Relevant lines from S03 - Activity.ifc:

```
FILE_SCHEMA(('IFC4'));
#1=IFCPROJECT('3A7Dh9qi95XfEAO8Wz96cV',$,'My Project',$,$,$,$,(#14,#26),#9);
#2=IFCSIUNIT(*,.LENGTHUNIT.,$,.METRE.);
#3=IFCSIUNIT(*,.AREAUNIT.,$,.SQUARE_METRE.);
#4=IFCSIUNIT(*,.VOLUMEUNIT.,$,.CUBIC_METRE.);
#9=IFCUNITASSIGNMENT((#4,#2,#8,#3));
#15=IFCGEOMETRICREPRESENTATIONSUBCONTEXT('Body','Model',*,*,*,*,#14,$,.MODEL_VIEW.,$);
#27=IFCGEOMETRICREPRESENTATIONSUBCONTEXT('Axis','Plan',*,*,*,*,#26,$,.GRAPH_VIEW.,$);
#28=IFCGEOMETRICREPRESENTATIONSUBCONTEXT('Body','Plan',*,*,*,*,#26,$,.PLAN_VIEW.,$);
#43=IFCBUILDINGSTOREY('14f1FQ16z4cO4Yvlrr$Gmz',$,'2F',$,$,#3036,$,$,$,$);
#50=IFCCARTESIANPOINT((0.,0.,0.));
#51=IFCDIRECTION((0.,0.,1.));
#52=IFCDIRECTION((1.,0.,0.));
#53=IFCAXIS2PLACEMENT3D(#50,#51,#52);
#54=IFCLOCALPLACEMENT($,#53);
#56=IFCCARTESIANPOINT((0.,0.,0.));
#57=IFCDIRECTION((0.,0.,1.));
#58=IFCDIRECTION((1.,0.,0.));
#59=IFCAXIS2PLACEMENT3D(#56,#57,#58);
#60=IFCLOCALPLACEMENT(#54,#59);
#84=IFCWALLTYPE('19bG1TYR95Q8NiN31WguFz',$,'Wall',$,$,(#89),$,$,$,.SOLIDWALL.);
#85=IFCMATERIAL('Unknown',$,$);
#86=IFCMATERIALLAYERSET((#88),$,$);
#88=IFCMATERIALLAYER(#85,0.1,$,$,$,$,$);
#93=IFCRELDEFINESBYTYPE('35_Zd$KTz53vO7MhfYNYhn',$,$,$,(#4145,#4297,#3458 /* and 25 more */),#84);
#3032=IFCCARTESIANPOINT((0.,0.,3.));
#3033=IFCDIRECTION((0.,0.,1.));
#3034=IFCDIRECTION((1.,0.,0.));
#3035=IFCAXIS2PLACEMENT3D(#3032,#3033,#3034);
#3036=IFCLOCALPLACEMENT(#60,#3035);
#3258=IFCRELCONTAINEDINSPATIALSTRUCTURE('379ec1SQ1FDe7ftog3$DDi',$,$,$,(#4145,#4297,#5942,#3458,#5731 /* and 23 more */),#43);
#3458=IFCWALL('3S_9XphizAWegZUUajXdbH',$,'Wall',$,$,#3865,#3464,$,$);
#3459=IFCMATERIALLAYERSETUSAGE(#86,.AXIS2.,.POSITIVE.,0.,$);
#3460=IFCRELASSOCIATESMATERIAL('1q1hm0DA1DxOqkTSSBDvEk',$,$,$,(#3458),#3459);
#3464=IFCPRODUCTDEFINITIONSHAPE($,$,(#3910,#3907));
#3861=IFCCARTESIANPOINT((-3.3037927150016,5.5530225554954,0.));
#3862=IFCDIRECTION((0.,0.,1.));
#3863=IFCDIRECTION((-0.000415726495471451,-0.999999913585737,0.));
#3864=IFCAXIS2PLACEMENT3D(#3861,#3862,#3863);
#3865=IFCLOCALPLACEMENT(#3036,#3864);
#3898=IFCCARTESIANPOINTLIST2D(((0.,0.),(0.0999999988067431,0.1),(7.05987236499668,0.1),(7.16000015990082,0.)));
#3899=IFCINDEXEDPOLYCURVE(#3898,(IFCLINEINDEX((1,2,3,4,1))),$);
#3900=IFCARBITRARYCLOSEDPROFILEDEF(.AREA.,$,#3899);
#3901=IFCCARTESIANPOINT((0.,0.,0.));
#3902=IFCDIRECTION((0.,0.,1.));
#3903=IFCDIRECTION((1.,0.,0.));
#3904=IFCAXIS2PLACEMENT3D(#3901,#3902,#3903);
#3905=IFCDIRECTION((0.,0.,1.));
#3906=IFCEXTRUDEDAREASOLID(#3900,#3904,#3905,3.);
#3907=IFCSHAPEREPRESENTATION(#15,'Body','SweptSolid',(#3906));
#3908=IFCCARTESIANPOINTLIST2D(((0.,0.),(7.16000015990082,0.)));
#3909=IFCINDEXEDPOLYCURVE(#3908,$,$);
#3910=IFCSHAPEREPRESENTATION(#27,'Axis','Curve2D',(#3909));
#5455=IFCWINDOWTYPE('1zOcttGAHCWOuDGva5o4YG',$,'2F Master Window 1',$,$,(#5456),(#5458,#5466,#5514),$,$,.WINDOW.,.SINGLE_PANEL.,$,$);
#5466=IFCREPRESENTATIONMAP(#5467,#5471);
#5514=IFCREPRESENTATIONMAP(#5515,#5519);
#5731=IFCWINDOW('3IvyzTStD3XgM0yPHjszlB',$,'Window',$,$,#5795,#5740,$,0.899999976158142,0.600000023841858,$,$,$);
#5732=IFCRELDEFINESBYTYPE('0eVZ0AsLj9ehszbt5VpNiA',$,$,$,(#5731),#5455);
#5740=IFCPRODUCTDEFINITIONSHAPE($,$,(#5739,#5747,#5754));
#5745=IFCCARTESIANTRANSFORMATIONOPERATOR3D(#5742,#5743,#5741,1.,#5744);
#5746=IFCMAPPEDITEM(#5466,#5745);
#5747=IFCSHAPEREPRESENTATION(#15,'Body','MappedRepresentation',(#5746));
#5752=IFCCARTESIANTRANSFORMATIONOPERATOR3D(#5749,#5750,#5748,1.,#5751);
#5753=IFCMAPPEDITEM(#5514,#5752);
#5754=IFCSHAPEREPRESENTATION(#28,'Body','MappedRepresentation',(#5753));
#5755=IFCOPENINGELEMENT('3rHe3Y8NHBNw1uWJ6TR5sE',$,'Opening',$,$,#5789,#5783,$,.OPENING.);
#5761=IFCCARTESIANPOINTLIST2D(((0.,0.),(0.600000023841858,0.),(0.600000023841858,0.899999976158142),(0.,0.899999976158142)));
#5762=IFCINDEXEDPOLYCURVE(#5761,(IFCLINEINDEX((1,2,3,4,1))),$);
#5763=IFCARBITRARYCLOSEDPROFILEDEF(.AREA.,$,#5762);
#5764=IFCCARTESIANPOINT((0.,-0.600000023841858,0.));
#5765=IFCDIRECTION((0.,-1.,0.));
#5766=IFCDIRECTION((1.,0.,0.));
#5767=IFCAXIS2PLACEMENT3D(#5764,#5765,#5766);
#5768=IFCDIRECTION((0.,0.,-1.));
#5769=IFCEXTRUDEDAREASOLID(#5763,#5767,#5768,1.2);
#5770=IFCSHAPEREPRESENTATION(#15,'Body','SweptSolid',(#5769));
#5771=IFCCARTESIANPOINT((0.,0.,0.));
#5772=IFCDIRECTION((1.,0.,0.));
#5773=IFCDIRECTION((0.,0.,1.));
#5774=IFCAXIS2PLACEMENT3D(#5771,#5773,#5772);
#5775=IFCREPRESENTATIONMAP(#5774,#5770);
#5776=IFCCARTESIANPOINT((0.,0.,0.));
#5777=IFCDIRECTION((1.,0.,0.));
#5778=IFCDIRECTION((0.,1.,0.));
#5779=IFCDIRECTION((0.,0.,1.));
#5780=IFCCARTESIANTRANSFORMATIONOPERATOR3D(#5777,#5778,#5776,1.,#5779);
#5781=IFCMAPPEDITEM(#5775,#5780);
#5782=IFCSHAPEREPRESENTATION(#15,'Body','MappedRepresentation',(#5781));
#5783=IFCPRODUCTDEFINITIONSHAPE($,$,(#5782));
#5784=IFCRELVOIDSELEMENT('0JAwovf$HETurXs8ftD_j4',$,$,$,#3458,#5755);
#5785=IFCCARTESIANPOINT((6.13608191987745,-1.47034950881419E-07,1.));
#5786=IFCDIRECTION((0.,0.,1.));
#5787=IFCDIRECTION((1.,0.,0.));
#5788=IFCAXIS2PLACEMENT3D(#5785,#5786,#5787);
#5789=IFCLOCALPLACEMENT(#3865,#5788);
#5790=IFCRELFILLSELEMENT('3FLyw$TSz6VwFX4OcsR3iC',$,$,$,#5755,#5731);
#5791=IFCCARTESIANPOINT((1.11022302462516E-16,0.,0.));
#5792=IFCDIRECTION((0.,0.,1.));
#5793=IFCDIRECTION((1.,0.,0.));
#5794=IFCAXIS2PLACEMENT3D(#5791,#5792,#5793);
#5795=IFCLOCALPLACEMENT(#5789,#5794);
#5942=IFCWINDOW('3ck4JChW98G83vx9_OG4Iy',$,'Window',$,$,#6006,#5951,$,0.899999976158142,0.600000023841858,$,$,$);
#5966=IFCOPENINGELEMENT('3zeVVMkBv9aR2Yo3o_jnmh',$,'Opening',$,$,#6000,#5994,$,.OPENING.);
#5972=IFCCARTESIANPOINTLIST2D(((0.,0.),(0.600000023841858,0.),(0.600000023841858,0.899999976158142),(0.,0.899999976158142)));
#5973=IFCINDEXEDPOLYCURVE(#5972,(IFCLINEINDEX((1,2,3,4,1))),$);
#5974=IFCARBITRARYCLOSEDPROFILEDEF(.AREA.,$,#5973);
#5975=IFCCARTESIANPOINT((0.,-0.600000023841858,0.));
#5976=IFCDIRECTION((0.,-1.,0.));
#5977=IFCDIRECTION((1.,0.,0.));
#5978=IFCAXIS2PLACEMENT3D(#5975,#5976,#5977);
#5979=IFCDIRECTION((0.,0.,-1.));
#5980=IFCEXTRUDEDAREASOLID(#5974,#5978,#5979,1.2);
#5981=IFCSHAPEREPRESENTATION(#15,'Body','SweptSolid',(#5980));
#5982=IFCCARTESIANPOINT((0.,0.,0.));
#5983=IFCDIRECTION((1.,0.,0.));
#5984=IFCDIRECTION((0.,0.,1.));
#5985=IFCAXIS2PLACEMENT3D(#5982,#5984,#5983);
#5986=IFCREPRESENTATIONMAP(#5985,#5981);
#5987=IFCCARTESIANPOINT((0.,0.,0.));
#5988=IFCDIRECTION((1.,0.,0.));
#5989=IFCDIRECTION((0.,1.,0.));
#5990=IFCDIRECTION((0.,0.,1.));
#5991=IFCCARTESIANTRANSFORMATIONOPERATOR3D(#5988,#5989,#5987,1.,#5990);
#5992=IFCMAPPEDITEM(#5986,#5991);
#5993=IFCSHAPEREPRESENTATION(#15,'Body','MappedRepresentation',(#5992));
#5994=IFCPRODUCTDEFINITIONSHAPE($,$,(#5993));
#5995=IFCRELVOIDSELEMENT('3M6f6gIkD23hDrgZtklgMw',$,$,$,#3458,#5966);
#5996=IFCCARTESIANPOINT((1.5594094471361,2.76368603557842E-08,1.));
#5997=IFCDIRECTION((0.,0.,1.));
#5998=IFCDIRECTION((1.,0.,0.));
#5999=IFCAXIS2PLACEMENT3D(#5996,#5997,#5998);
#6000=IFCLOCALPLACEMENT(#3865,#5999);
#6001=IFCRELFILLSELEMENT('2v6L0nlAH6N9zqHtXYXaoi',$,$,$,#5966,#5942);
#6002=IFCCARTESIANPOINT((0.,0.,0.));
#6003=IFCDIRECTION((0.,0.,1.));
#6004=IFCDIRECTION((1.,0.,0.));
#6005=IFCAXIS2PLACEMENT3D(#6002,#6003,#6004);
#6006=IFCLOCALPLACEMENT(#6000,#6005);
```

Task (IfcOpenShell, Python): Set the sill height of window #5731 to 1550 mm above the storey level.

```python
import numpy as np
import ifcopenshell
import ifcopenshell.api.geometry
import ifcopenshell.geom
import ifcopenshell.util.element
import ifcopenshell.util.placement
import ifcopenshell.util.shape
import ifcopenshell.util.unit

model = ifcopenshell.open("S03 - Activity.ifc")
unit_scale = ifcopenshell.util.unit.calculate_unit_scale(model)

window = model.by_guid("3IvyzTStD3XgM0yPHjszlB")
opening = window.FillsVoids[0].RelatingOpeningElement
storey = ifcopenshell.util.element.get_container(window, ifc_class="IfcBuildingStorey")
level = ifcopenshell.util.placement.get_local_placement(storey.ObjectPlacement)[2, 3]

# The opening's origin need not be at the sill, so measure its lowest point.
shape = ifcopenshell.geom.create_shape(ifcopenshell.geom.settings(), opening)
bottom = ifcopenshell.util.shape.get_shape_bottom_elevation(shape, shape.geometry) / unit_scale
dz = level + 1.55 - bottom

shift = np.array([0.0, 0.0, dz])
# The window is placed relative to its opening, so it follows when the opening moves.
matrix = ifcopenshell.util.placement.get_local_placement(opening.ObjectPlacement)
matrix[:3, 3] += shift
ifcopenshell.api.geometry.edit_object_placement(
    model, product=opening, matrix=matrix, is_si=False, should_transform_children=True
)

print(f"moved by {dz * unit_scale:+.3f} m")

model.write("S03 - Activity_v2.ifc")
```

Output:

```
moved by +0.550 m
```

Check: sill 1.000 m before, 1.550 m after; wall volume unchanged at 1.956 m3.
